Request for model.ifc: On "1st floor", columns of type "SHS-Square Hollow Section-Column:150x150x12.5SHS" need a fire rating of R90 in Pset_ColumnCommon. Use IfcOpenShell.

First a look at what the model holds.

```python
import ifcopenshell
import ifcopenshell.util.element

model = ifcopenshell.open("model.ifc")
print(model.schema)
storey = next(s for s in model.by_type("IfcBuildingStorey") if s.Name == "1st floor")
columns = [e for e in ifcopenshell.util.element.get_decomposition(storey) if e.is_a("IfcColumn")]
seen = {}
for e in columns:
    element_type = ifcopenshell.util.element.get_type(e)
    key = (element_type.Name if element_type != e and element_type else None, ifcopenshell.util.element.get_pset(e, "Pset_ColumnCommon", "FireRating"))
    seen[key] = seen.get(key, 0) + 1
for (name, value), count in sorted(seen.items(), key=str):
    print(count, "x", name, "|", value)
```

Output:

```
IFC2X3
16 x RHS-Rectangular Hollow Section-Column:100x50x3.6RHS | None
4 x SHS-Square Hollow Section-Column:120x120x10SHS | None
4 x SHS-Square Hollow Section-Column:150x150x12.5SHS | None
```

```python
import ifcopenshell
import ifcopenshell.api.pset
import ifcopenshell.util.element

model = ifcopenshell.open("model.ifc")

storey = next(s for s in model.by_type("IfcBuildingStorey") if s.Name == "1st floor")
columns = [e for e in ifcopenshell.util.element.get_decomposition(storey) if e.is_a("IfcColumn")]

count = 0
for e in columns:
    element_type = ifcopenshell.util.element.get_type(e)
    if element_type in (None, e) or element_type.Name != "SHS-Square Hollow Section-Column:150x150x12.5SHS":
        continue
    # add_pset returns the element's existing set when there is one.
    pset = ifcopenshell.api.pset.add_pset(model, product=e, name="Pset_ColumnCommon")
    ifcopenshell.api.pset.edit_pset(model, pset=pset, properties={"FireRating": "R90"})
    count += 1

print(count, "columns updated")

model.write("model-out.ifc")
```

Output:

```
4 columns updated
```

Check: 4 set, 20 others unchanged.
